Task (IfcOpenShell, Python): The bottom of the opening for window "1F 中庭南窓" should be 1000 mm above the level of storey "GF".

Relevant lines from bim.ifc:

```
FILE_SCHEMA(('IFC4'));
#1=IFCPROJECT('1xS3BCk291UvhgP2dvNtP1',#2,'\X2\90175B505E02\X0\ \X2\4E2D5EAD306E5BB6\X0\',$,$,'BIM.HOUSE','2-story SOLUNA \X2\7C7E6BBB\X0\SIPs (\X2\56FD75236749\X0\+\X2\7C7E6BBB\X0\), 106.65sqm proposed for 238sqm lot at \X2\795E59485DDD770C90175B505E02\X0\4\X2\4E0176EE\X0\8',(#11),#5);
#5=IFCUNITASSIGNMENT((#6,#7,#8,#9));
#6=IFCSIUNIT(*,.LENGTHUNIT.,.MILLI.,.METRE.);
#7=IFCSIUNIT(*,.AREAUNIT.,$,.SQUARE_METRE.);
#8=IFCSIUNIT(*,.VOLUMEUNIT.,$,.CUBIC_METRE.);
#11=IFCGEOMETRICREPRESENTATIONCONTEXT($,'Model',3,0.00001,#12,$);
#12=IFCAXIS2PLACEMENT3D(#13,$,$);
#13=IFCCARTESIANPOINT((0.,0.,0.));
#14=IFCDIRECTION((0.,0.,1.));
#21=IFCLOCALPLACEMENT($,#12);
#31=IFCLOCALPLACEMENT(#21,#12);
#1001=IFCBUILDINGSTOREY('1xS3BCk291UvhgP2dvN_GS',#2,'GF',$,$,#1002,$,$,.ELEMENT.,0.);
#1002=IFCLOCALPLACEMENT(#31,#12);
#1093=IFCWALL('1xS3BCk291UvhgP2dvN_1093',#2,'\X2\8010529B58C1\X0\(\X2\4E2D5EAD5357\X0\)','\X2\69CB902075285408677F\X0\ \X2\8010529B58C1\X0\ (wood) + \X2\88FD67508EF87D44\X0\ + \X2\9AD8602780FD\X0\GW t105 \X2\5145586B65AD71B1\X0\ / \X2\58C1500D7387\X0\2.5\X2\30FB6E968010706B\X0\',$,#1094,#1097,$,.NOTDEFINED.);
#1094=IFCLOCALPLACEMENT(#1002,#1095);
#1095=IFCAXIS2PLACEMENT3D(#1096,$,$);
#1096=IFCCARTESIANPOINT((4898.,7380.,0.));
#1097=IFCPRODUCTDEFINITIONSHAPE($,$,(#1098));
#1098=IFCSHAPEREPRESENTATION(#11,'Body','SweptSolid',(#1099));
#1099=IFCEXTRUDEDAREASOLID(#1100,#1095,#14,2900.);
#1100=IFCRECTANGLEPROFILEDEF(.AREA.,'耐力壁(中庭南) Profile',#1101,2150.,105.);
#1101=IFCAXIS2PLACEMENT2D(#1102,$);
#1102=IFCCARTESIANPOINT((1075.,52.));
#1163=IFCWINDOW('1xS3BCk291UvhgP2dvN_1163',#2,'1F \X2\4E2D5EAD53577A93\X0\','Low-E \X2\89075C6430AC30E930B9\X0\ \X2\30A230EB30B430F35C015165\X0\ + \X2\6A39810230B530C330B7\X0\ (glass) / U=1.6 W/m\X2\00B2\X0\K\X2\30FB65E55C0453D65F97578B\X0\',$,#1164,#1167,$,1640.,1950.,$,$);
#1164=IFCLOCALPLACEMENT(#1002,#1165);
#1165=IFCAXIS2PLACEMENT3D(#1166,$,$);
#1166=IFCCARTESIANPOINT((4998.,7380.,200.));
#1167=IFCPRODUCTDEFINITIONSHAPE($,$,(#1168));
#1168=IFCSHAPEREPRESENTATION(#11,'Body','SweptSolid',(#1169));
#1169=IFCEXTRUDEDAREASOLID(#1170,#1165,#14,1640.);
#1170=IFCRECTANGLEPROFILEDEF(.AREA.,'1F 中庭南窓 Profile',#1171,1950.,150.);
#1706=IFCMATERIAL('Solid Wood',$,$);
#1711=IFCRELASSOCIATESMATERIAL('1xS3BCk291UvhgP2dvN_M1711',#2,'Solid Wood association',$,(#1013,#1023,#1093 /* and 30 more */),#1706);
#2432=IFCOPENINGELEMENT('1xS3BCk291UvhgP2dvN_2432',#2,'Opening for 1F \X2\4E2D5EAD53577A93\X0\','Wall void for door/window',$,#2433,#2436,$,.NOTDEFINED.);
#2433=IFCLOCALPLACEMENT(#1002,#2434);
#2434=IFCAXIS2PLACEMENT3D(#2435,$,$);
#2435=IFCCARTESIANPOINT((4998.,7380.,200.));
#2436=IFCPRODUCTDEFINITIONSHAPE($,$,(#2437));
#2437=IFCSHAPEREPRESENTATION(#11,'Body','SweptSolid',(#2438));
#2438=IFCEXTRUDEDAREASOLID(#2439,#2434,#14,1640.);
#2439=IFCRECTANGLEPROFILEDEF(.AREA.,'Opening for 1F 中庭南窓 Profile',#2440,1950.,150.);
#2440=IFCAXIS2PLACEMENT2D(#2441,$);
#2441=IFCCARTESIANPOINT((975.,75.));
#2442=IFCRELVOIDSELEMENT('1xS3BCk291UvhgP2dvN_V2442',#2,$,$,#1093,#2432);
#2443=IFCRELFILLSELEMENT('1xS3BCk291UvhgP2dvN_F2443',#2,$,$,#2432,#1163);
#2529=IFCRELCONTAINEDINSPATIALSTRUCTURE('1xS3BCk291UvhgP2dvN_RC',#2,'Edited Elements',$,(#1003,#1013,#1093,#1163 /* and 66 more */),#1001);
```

```python
import numpy as np
import ifcopenshell
import ifcopenshell.api.geometry
import ifcopenshell.geom
import ifcopenshell.util.element
import ifcopenshell.util.placement
import ifcopenshell.util.shape
import ifcopenshell.util.unit

model = ifcopenshell.open("bim.ifc")
unit_scale = ifcopenshell.util.unit.calculate_unit_scale(model)

window = model.by_id(1163)
opening = window.FillsVoids[0].RelatingOpeningElement
storey = ifcopenshell.util.element.get_container(window, ifc_class="IfcBuildingStorey")
level = ifcopenshell.util.placement.get_local_placement(storey.ObjectPlacement)[2, 3]

# The opening's origin need not be at the sill, so measure its lowest point.
shape = ifcopenshell.geom.create_shape(ifcopenshell.geom.settings(), opening)
bottom = ifcopenshell.util.shape.get_shape_bottom_elevation(shape, shape.geometry) / unit_scale
dz = level + 1000.0 - bottom

shift = np.array([0.0, 0.0, dz])
# The window is not placed relative to its opening, so move both.
for product in (opening, window):
    matrix = ifcopenshell.util.placement.get_local_placement(product.ObjectPlacement)
    matrix[:3, 3] += shift
    ifcopenshell.api.geometry.edit_object_placement(model, product=product, matrix=matrix, is_si=False)

print(f"moved by {dz * unit_scale:+.3f} m")

model.write("bim_updated.ifc")
```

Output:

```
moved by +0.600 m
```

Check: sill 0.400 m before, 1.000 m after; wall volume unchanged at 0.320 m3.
